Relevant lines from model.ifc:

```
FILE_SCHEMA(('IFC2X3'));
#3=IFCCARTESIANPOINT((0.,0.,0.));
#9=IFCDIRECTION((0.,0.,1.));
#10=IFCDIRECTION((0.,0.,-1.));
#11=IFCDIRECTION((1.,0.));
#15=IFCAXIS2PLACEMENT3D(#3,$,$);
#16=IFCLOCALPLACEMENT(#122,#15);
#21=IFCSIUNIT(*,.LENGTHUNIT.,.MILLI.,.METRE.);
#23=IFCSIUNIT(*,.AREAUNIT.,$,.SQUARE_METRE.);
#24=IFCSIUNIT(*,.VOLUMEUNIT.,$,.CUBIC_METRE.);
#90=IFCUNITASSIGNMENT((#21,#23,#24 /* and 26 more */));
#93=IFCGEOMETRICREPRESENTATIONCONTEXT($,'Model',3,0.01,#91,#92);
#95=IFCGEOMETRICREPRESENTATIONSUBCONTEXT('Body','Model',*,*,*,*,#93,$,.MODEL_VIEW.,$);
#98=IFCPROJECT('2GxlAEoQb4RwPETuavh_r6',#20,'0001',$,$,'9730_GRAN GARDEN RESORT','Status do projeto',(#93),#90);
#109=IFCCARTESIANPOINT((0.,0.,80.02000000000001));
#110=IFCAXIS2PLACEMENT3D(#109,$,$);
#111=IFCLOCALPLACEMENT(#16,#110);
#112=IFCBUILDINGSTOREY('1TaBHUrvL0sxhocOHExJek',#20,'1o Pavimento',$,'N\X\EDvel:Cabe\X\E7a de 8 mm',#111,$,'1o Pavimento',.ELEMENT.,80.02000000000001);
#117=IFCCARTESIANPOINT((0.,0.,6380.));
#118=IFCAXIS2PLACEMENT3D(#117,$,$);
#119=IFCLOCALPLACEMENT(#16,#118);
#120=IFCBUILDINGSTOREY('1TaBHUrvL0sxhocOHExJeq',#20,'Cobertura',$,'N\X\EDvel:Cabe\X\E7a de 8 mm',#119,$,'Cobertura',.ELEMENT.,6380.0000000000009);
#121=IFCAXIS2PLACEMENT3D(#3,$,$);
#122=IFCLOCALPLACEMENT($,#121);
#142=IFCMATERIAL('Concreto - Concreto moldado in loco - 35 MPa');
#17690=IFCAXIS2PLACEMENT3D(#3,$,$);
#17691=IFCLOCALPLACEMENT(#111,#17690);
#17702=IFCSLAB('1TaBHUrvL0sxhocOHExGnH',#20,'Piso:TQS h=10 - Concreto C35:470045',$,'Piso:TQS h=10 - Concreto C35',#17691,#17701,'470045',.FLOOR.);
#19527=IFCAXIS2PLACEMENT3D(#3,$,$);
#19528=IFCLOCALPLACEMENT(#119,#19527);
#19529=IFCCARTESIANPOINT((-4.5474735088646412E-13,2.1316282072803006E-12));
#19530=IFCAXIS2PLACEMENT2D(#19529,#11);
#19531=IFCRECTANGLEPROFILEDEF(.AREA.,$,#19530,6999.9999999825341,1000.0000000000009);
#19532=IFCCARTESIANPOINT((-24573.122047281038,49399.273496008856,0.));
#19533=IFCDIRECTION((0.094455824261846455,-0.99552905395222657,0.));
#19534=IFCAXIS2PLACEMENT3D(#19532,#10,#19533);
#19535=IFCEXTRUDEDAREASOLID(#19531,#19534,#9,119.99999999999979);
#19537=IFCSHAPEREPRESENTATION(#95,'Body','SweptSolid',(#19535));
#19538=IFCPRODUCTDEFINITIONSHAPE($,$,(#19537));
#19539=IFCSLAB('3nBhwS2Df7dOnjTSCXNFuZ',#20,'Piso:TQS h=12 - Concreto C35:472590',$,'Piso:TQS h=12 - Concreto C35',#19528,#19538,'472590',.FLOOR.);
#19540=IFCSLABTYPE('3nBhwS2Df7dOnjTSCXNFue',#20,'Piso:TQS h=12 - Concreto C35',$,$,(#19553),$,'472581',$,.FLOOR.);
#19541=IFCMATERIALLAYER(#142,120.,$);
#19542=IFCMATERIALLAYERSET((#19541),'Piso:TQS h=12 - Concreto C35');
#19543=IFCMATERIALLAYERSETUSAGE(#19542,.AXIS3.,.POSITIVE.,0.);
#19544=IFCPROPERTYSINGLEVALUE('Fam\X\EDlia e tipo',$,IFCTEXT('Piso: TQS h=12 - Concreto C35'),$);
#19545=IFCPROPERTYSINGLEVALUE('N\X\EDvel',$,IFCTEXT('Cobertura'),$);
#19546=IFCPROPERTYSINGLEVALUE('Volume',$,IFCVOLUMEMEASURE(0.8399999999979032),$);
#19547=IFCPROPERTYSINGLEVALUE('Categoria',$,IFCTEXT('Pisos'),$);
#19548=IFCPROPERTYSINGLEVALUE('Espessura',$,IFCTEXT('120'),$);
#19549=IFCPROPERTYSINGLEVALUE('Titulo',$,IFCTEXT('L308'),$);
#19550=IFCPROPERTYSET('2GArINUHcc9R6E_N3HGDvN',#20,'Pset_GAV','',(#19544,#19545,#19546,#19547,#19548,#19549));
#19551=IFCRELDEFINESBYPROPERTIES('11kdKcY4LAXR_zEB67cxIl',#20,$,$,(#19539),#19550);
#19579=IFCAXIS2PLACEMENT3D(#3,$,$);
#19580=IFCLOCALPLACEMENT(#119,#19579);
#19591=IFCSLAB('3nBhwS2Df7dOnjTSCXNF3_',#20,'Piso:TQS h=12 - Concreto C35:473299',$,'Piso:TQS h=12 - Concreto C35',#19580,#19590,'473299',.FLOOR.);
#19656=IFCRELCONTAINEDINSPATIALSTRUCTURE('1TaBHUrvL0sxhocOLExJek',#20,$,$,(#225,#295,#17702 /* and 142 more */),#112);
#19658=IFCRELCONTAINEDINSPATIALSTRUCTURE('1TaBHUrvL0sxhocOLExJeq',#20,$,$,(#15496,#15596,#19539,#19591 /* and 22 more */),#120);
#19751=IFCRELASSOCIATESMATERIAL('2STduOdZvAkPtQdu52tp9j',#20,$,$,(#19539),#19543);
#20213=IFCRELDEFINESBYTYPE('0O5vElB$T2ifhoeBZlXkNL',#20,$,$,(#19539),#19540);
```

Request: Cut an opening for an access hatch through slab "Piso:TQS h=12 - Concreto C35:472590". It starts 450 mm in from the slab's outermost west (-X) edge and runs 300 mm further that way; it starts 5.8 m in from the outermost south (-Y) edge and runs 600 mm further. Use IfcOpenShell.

```python
import numpy as np
import ifcopenshell
import ifcopenshell.api.feature
import ifcopenshell.api.geometry
import ifcopenshell.api.pset
import ifcopenshell.api.root
import ifcopenshell.geom
import ifcopenshell.util.element
import ifcopenshell.util.placement
import ifcopenshell.util.representation
import ifcopenshell.util.shape
import ifcopenshell.util.unit

model = ifcopenshell.open("model.ifc")
unit_scale = ifcopenshell.util.unit.calculate_unit_scale(model)
volume_scale = ifcopenshell.util.unit.calculate_unit_scale(model, "VOLUMEUNIT")
settings = ifcopenshell.geom.settings()


def volume(element):
    """Net volume in cubic metres, openings subtracted."""
    shape = ifcopenshell.geom.create_shape(settings, element)
    return ifcopenshell.util.shape.get_volume(shape.geometry)


slab = model.by_guid("3nBhwS2Df7dOnjTSCXNFuZ")
before = volume(slab)

# Extent in the slab's own axes, in metres. The edges named are its -X and -Y sides.
slab_shape = ifcopenshell.geom.create_shape(settings, slab)
vertices = ifcopenshell.util.shape.get_vertices(slab_shape.geometry)
x_min, y_min, bottom = vertices.min(axis=0)
top = vertices[:, 2].max()

opening = ifcopenshell.api.root.create_entity(model, ifc_class="IfcOpeningElement", name="Access hatch opening")
context = ifcopenshell.util.representation.get_context(model, "Model", "Body", "MODEL_VIEW")
width, depth = 0.3, 0.6
outline = [(0.0, 0.0), (width, 0.0), (width, depth), (0.0, depth), (0.0, 0.0)]
# Overshoot both faces by 50 mm so the cut is clean.
shape = ifcopenshell.api.geometry.add_slab_representation(
    model, context=context, depth=top - bottom + 0.1, polyline=outline
)
ifcopenshell.api.geometry.assign_representation(model, product=opening, representation=shape)

matrix = ifcopenshell.util.placement.get_local_placement(slab.ObjectPlacement)
matrix[:, 3] = matrix @ np.append(np.array([x_min + 0.45, y_min + 5.8, bottom - 0.05]) / unit_scale, 1.0)
ifcopenshell.api.geometry.edit_object_placement(model, product=opening, matrix=matrix, is_si=False)
ifcopenshell.api.feature.add_feature(model, feature=opening, element=slab)

after = volume(slab)

# Update the slab's stored quantities.
pset = model.by_id(ifcopenshell.util.element.get_pset(slab, "Pset_GAV", should_inherit=False)["id"])
ifcopenshell.api.pset.edit_pset(model, pset=pset, properties={
    "Volume": model.create_entity("IfcVolumeMeasure", after / volume_scale),
})

print(f"slab volume {before:.3f} -> {after:.3f} m3")

model.write("model-out.ifc")
```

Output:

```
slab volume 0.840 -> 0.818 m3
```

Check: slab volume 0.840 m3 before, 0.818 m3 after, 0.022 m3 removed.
